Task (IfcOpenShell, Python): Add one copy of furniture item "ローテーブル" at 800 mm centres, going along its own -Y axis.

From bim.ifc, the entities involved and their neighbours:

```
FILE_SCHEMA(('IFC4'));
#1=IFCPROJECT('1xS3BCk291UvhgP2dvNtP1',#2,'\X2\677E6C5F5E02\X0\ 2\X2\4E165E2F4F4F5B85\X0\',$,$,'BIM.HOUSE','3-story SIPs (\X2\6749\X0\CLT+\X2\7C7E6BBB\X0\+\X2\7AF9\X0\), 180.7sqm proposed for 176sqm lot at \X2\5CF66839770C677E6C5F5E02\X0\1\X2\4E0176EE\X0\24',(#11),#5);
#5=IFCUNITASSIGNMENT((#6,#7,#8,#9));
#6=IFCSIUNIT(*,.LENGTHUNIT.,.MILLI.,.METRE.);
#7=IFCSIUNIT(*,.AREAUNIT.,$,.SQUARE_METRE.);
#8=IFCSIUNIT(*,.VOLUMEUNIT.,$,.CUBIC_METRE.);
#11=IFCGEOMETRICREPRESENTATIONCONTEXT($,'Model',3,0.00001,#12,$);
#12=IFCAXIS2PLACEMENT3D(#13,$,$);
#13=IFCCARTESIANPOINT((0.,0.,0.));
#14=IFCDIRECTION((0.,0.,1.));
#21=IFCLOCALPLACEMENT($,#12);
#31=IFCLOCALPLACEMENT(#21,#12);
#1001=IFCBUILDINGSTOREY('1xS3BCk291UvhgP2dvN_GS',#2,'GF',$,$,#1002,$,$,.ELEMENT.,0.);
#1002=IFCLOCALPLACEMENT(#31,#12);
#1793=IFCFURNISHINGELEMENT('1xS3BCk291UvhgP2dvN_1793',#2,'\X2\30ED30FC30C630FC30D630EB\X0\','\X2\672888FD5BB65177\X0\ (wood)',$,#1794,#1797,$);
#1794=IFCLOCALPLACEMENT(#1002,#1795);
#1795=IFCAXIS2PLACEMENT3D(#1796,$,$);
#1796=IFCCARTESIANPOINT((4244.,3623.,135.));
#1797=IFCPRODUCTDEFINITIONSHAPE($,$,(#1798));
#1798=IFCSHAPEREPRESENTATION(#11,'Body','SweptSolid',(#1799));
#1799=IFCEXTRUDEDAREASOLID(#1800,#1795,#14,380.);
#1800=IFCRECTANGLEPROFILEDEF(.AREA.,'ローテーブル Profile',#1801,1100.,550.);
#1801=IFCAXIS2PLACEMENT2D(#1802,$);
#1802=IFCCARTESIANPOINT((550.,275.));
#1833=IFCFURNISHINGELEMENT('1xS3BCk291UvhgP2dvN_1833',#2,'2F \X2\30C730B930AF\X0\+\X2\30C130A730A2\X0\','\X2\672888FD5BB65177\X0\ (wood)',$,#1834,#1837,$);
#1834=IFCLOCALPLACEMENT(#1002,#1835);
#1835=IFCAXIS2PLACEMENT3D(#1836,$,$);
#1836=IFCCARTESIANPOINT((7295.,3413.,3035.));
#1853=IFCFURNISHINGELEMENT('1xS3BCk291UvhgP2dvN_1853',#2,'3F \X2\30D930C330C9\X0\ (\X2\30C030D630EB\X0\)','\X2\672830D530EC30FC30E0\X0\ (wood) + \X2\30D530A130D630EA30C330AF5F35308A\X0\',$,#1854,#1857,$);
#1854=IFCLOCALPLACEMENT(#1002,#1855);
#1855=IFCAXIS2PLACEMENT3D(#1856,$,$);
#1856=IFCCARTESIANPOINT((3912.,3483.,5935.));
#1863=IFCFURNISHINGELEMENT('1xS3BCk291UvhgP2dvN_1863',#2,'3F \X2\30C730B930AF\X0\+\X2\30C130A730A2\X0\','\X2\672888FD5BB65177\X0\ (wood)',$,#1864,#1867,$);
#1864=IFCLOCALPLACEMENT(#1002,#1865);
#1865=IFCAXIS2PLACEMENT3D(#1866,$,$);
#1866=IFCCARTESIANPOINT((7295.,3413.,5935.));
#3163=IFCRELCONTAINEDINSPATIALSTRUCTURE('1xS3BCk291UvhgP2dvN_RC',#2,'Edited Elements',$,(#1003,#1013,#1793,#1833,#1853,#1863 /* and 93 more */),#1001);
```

```python
import ifcopenshell
import ifcopenshell.api.geometry
import ifcopenshell.api.root
import ifcopenshell.util.element
import ifcopenshell.util.placement
import ifcopenshell.util.unit

model = ifcopenshell.open("bim.ifc")
unit_scale = ifcopenshell.util.unit.calculate_unit_scale(model)


def reuse_history(source, copy):
    """copy_class also copies each property set's owner history, people and application; keep the originals."""
    for rel in copy.IsDefinedBy:
        if rel.is_a("IfcRelDefinesByProperties") and (history := rel.RelatingPropertyDefinition.OwnerHistory):
            rel.RelatingPropertyDefinition.OwnerHistory = source.OwnerHistory
            ifcopenshell.util.element.remove_deep2(model, history)


source = model.by_guid("1xS3BCk291UvhgP2dvN_1793")
base = ifcopenshell.util.placement.get_local_placement(source.ObjectPlacement)
step = -base[:3, 1] * 0.8 / unit_scale

for i in range(1, 2):
    copy = ifcopenshell.api.root.copy_class(model, product=source)
    copy.Representation = ifcopenshell.util.element.copy_deep(
        model, source.Representation, exclude=["IfcGeometricRepresentationContext", "IfcRepresentationMap"]
    )
    reuse_history(source, copy)
    matrix = base.copy()
    matrix[:3, 3] += i * step
    print("added at", matrix[:3, 3].round(3) + 0.0)
    ifcopenshell.api.geometry.edit_object_placement(model, product=copy, matrix=matrix, is_si=False)

model.write("bim_updated.ifc")
```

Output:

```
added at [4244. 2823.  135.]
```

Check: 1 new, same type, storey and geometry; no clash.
